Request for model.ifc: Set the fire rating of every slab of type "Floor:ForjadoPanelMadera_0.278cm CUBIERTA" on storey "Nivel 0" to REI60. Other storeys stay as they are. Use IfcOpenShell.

First a look at what the model holds.

```python
import ifcopenshell
import ifcopenshell.util.element

model = ifcopenshell.open("model.ifc")
print(model.schema)
storey = next(s for s in model.by_type("IfcBuildingStorey") if s.Name == "Nivel 0")
slabs = [e for e in ifcopenshell.util.element.get_decomposition(storey) if e.is_a("IfcSlab")]
seen = {}
for e in slabs:
    element_type = ifcopenshell.util.element.get_type(e)
    key = (element_type.Name if element_type != e and element_type else None, ifcopenshell.util.element.get_pset(e, "Pset_SlabCommon", "FireRating"))
    seen[key] = seen.get(key, 0) + 1
for (name, value), count in sorted(seen.items(), key=str):
    print(count, "x", name, "|", value)
```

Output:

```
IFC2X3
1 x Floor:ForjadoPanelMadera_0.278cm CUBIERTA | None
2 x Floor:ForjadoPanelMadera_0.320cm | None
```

```python
import ifcopenshell
import ifcopenshell.api.pset
import ifcopenshell.util.element

model = ifcopenshell.open("model.ifc")

storey = next(s for s in model.by_type("IfcBuildingStorey") if s.Name == "Nivel 0")
slabs = [e for e in ifcopenshell.util.element.get_decomposition(storey) if e.is_a("IfcSlab")]

count = 0
for e in slabs:
    element_type = ifcopenshell.util.element.get_type(e)
    if element_type in (None, e) or element_type.Name != "Floor:ForjadoPanelMadera_0.278cm CUBIERTA":
        continue
    # add_pset returns the element's existing set when there is one.
    pset = ifcopenshell.api.pset.add_pset(model, product=e, name="Pset_SlabCommon")
    ifcopenshell.api.pset.edit_pset(model, pset=pset, properties={"FireRating": "REI60"})
    count += 1

print(count, "slabs updated")

model.write("model_updated.ifc")
```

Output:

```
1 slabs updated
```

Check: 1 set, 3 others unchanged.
